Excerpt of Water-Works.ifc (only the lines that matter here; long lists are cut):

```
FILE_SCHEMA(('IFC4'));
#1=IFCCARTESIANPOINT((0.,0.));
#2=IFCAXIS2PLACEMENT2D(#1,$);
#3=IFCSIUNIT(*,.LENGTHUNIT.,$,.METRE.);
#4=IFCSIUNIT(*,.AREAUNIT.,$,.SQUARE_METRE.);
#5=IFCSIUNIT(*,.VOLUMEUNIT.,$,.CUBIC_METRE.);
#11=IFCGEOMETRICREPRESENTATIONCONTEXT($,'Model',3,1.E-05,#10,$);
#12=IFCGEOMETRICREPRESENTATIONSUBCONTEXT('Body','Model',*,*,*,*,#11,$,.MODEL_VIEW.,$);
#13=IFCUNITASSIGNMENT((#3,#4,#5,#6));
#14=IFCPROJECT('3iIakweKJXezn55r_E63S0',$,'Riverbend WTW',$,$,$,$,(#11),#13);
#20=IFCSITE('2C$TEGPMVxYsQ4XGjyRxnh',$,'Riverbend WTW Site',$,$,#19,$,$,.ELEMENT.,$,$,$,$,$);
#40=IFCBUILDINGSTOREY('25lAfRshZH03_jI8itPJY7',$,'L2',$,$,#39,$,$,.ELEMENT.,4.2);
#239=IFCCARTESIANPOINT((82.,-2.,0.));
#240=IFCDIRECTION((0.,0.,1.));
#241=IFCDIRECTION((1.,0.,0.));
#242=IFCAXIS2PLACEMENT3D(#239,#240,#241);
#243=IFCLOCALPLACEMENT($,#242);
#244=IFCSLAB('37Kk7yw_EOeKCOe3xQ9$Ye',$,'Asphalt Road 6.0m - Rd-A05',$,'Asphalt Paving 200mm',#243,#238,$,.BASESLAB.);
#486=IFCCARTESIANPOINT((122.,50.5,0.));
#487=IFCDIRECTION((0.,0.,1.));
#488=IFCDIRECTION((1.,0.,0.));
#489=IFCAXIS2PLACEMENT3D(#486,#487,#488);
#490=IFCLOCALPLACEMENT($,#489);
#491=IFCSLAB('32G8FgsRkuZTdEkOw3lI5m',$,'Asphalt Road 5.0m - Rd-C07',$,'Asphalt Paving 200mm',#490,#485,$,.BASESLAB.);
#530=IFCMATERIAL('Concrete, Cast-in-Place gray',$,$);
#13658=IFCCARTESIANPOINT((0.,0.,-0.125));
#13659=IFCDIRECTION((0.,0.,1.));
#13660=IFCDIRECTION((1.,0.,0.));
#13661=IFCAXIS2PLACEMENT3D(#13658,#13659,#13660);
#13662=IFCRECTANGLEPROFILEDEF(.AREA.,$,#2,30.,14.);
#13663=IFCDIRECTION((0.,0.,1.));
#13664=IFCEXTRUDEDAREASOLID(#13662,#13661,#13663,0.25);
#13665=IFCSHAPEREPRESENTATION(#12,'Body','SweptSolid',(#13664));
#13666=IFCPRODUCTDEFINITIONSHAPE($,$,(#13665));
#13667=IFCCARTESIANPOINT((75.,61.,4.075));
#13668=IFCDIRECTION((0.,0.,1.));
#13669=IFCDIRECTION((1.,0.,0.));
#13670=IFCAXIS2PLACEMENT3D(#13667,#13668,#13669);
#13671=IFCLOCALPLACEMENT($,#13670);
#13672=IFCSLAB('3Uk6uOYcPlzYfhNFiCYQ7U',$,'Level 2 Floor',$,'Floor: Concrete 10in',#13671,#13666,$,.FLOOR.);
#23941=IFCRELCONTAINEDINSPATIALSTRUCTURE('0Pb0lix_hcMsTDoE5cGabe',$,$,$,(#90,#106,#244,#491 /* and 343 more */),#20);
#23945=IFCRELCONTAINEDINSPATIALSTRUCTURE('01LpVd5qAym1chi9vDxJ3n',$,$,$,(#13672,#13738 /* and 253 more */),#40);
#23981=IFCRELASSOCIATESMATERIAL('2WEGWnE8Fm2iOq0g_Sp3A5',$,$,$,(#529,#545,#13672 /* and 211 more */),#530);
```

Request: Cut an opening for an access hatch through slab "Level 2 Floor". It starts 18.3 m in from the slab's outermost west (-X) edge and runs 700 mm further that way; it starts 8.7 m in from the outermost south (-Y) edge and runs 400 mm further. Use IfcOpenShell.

```python
import numpy as np
import ifcopenshell
import ifcopenshell.api.feature
import ifcopenshell.api.geometry
import ifcopenshell.api.root
import ifcopenshell.geom
import ifcopenshell.util.placement
import ifcopenshell.util.representation
import ifcopenshell.util.shape
import ifcopenshell.util.unit

model = ifcopenshell.open("Water-Works.ifc")
unit_scale = ifcopenshell.util.unit.calculate_unit_scale(model)
settings = ifcopenshell.geom.settings()


def volume(element):
    """Net volume in cubic metres, openings subtracted."""
    shape = ifcopenshell.geom.create_shape(settings, element)
    return ifcopenshell.util.shape.get_volume(shape.geometry)


slab = model.by_guid("3Uk6uOYcPlzYfhNFiCYQ7U")
before = volume(slab)

# Extent in the slab's own axes, in metres. The edges named are its -X and -Y sides.
slab_shape = ifcopenshell.geom.create_shape(settings, slab)
vertices = ifcopenshell.util.shape.get_vertices(slab_shape.geometry)
x_min, y_min, bottom = vertices.min(axis=0)
top = vertices[:, 2].max()

opening = ifcopenshell.api.root.create_entity(model, ifc_class="IfcOpeningElement", name="Access hatch opening", predefined_type="OPENING")
context = ifcopenshell.util.representation.get_context(model, "Model", "Body", "MODEL_VIEW")
width, depth = 0.7, 0.4
outline = [(0.0, 0.0), (width, 0.0), (width, depth), (0.0, depth), (0.0, 0.0)]
# Overshoot both faces by 50 mm so the cut is clean.
shape = ifcopenshell.api.geometry.add_slab_representation(
    model, context=context, depth=top - bottom + 0.1, polyline=outline
)
ifcopenshell.api.geometry.assign_representation(model, product=opening, representation=shape)

matrix = ifcopenshell.util.placement.get_local_placement(slab.ObjectPlacement)
matrix[:, 3] = matrix @ np.append(np.array([x_min + 18.3, y_min + 8.7, bottom - 0.05]) / unit_scale, 1.0)
ifcopenshell.api.geometry.edit_object_placement(model, product=opening, matrix=matrix, is_si=False)
ifcopenshell.api.feature.add_feature(model, feature=opening, element=slab)

after = volume(slab)

print(f"slab volume {before:.3f} -> {after:.3f} m3")

model.write("Water-Works_rev.ifc")
```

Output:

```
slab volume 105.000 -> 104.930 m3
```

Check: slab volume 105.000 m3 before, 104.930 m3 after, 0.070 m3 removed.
